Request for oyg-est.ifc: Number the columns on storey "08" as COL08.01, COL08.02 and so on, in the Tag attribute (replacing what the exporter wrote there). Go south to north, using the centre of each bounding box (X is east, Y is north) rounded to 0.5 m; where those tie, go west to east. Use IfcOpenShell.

First a look at what the model holds.

```python
import ifcopenshell
import ifcopenshell.util.element
import ifcopenshell.util.placement

model = ifcopenshell.open("oyg-est.ifc")
print(model.schema)
storey = next(s for s in model.by_type("IfcBuildingStorey") if s.Name == "08")
columns = [e for e in ifcopenshell.util.element.get_decomposition(storey) if e.is_a("IfcColumn")]
for e in sorted(columns, key=lambda e: e.id()):
    origin = ifcopenshell.util.placement.get_local_placement(e.ObjectPlacement)[:3, 3]
    print(e.id(), e.Tag, e.Name, origin.round(2) + 0.0, sep=" | ")
```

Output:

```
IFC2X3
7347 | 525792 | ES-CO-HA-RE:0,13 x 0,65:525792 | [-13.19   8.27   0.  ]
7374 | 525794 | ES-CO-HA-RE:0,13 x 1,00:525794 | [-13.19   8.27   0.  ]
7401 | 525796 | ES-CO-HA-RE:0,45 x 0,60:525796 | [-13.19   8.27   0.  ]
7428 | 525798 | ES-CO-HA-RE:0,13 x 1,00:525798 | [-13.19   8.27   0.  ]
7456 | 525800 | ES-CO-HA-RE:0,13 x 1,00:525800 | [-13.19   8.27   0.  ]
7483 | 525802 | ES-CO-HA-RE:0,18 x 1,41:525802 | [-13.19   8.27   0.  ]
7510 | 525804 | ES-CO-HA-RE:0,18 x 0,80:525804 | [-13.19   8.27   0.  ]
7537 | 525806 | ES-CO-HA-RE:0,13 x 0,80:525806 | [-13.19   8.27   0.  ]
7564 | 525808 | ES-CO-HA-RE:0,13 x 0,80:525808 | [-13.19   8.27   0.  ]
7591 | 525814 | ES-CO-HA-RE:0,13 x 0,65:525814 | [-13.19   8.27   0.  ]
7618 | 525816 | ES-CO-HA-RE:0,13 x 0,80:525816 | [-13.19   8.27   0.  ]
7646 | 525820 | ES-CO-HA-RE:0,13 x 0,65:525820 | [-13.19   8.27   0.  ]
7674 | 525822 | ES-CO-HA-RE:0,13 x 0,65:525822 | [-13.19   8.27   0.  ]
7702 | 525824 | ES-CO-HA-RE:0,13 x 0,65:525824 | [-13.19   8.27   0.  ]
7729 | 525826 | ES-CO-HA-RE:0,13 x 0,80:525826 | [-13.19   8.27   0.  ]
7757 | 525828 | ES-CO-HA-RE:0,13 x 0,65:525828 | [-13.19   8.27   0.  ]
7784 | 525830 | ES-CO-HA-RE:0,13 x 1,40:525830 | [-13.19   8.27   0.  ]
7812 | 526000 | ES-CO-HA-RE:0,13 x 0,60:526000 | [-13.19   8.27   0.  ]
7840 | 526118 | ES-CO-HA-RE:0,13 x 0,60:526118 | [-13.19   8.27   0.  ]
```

```python
import ifcopenshell
import ifcopenshell.geom
import ifcopenshell.util.element
import ifcopenshell.util.shape

model = ifcopenshell.open("oyg-est.ifc")
settings = ifcopenshell.geom.settings()
settings.set("use-world-coords", True)


def centre(element):
    shape = ifcopenshell.geom.create_shape(settings, element)
    return ifcopenshell.util.shape.get_bbox_centroid(shape.geometry)


storey = next(s for s in model.by_type("IfcBuildingStorey") if s.Name == "08")
columns = [e for e in ifcopenshell.util.element.get_decomposition(storey) if e.is_a("IfcColumn")]

# Insertion points can sit at a corner or the storey origin, so sort by the geometry (in metres).
centres = {e: centre(e) for e in columns}
columns.sort(key=lambda e: (round(centres[e][1] / 0.5), centres[e][0]))

for i, e in enumerate(columns, start=1):
    number = f"COL08.{i:02d}"
    e.Tag = number
    print(e.id(), number)

model.write("oyg-est_updated.ifc")
```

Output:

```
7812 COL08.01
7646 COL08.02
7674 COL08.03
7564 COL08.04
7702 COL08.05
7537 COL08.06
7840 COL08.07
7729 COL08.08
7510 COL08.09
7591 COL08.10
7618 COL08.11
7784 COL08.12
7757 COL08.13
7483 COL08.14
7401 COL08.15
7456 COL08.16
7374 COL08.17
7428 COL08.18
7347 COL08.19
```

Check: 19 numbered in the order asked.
